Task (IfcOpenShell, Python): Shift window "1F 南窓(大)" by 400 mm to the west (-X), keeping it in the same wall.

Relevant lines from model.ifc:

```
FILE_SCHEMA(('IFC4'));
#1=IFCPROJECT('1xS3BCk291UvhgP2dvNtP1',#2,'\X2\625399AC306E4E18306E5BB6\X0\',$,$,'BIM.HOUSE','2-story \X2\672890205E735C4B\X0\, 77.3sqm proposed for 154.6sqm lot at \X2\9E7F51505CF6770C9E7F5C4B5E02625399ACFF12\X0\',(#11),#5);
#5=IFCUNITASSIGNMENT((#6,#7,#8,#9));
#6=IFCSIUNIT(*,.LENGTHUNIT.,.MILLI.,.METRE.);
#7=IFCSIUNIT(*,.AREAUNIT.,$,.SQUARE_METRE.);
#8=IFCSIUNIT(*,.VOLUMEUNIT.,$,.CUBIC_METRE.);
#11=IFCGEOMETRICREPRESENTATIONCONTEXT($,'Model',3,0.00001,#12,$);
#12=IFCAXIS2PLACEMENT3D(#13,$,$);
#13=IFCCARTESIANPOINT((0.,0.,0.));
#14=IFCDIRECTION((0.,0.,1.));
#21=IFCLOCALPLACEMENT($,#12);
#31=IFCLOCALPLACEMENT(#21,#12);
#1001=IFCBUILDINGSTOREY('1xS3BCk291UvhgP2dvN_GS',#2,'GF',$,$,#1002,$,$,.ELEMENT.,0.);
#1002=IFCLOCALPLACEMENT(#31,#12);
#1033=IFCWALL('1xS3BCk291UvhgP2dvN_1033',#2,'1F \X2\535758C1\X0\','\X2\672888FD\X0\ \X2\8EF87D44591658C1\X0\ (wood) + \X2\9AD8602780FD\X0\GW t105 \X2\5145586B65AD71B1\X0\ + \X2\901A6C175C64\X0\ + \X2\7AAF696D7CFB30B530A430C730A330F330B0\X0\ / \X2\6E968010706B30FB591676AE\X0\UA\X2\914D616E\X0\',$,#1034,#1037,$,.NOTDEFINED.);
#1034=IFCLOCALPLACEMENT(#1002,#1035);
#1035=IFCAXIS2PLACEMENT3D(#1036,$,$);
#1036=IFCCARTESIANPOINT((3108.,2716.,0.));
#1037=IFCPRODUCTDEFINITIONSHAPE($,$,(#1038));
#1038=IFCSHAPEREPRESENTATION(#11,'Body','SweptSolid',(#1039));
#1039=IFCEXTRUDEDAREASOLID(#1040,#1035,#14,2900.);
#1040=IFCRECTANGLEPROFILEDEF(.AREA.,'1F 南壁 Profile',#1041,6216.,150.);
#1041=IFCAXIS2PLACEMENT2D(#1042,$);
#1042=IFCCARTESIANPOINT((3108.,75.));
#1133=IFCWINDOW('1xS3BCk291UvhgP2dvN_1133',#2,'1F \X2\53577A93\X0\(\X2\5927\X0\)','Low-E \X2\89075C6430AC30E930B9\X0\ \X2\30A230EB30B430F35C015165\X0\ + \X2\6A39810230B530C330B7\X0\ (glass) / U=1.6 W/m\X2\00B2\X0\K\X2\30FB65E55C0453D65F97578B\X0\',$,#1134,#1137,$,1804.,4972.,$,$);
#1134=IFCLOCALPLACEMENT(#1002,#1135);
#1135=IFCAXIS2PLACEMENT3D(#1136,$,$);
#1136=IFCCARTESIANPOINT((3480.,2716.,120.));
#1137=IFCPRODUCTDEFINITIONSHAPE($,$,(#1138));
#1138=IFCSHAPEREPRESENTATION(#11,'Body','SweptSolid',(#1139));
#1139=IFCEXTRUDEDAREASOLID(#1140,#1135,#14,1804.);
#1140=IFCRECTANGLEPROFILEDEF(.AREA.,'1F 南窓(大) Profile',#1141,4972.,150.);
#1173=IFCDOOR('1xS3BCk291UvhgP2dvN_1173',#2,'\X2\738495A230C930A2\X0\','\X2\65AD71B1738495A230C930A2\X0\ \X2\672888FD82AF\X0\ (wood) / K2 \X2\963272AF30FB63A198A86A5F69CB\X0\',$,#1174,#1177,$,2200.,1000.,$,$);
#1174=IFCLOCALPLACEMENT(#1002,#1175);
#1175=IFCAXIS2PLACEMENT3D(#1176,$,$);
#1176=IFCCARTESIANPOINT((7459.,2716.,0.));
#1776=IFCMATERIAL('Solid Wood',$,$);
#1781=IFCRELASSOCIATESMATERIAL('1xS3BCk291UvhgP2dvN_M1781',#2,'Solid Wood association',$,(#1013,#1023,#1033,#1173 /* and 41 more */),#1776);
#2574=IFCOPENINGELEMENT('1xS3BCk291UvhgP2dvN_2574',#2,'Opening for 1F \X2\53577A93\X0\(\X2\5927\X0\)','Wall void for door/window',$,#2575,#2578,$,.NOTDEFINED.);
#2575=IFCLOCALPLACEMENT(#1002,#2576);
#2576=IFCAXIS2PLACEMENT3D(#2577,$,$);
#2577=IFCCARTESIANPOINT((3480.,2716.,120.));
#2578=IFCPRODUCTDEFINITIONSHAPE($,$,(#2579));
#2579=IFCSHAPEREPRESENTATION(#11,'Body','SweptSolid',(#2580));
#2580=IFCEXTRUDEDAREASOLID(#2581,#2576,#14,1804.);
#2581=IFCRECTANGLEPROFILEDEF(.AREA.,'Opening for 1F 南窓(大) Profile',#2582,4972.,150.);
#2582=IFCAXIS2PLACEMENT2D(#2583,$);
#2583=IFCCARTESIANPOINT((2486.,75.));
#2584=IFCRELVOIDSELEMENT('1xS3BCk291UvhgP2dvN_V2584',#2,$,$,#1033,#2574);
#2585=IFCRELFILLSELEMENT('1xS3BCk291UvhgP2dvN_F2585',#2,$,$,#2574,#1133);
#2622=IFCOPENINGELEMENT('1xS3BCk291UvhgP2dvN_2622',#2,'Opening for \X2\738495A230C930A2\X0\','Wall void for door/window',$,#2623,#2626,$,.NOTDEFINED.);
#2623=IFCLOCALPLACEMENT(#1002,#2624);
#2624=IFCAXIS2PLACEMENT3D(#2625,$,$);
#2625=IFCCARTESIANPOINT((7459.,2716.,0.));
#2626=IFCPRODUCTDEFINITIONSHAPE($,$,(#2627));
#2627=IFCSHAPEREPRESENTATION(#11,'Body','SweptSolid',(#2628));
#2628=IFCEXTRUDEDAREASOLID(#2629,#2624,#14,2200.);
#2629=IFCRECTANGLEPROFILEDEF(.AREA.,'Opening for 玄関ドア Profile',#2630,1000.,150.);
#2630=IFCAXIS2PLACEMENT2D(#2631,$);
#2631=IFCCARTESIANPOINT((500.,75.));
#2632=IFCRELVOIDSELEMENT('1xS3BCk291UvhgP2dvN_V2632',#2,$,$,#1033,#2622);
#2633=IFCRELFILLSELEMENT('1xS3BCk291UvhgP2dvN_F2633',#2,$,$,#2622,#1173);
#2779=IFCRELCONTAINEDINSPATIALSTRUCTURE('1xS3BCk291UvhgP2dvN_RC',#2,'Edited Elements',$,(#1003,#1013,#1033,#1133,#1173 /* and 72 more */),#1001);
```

```python
import ifcopenshell
import ifcopenshell.api.geometry
import ifcopenshell.util.placement
import ifcopenshell.util.unit

model = ifcopenshell.open("model.ifc")
unit_scale = ifcopenshell.util.unit.calculate_unit_scale(model)

window = model.by_guid("1xS3BCk291UvhgP2dvN_1133")
opening = window.FillsVoids[0].RelatingOpeningElement
wall = opening.VoidsElements[0].RelatingBuildingElement

wall_matrix = ifcopenshell.util.placement.get_local_placement(wall.ObjectPlacement)
shift = wall_matrix[:3, 0] * -0.4 / unit_scale
before = ifcopenshell.util.placement.get_local_placement(window.ObjectPlacement)[:3, 3].copy()

# The window is not placed relative to its opening, so move both.
for product in (opening, window):
    matrix = ifcopenshell.util.placement.get_local_placement(product.ObjectPlacement)
    matrix[:3, 3] += shift
    ifcopenshell.api.geometry.edit_object_placement(model, product=product, matrix=matrix, is_si=False)

after = ifcopenshell.util.placement.get_local_placement(window.ObjectPlacement)[:3, 3]
print("window moved by", (after - before).round(3) + 0.0)

model.write("model-out.ifc")
```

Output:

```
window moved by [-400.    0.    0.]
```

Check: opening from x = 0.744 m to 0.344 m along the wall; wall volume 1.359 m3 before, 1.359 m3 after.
